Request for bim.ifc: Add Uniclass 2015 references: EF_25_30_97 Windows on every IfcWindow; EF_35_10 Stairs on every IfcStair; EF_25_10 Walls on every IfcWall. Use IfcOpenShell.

First a look at what the model holds.

```python
import ifcopenshell

model = ifcopenshell.open("bim.ifc")
print(model.schema)
print("classifications:", [c.Name for c in model.by_type("IfcClassification")])
for ifc_class in ("IfcDoor", "IfcRoof", "IfcStair", "IfcWall", "IfcWindow"):
    print(ifc_class, len(model.by_type(ifc_class)))
```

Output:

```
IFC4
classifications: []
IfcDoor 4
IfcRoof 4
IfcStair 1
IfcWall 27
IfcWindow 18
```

```python
import ifcopenshell
import ifcopenshell.api.classification

model = ifcopenshell.open("bim.ifc")

system = ifcopenshell.api.classification.add_classification(model, classification="Uniclass 2015")

codes = {
    "IfcWindow": ("EF_25_30_97", "Windows"),
    "IfcStair": ("EF_35_10", "Stairs"),
    "IfcWall": ("EF_25_10", "Walls"),
}
for ifc_class, (code, name) in codes.items():
    products = model.by_type(ifc_class)
    ifcopenshell.api.classification.add_reference(
        model, products=products, classification=system, identification=code, name=name
    )
    print(code, len(products))

model.write("bim-out.ifc")
```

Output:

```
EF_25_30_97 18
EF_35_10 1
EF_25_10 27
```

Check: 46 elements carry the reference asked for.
